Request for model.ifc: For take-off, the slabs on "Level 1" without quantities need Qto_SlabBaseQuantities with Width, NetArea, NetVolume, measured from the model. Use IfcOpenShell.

First a look at what the model holds.

```python
import ifcopenshell
import ifcopenshell.util.element
import ifcopenshell.util.unit

model = ifcopenshell.open("model.ifc")
print(model.schema)
for unit_type in ("LENGTHUNIT", "AREAUNIT", "VOLUMEUNIT"):
    print(unit_type, ifcopenshell.util.unit.calculate_unit_scale(model, unit_type))
storey = next(s for s in model.by_type("IfcBuildingStorey") if s.Name == "Level 1")
slabs = [e for e in ifcopenshell.util.element.get_decomposition(storey) if e.is_a("IfcSlab")]
for e in sorted(slabs, key=lambda e: e.id()):
    print(e.id(), e.is_a(), e.Name, list(ifcopenshell.util.element.get_psets(e, qtos_only=True)), sep=" | ")
```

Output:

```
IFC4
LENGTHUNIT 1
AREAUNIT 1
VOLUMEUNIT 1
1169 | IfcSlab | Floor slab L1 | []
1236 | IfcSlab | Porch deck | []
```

```python
import ifcopenshell
import ifcopenshell.api.pset
import ifcopenshell.geom
import ifcopenshell.util.element
import ifcopenshell.util.shape
import ifcopenshell.util.unit

model = ifcopenshell.open("model.ifc")
unit_scale = ifcopenshell.util.unit.calculate_unit_scale(model)
area_scale = ifcopenshell.util.unit.calculate_unit_scale(model, "AREAUNIT")
volume_scale = ifcopenshell.util.unit.calculate_unit_scale(model, "VOLUMEUNIT")
settings = ifcopenshell.geom.settings()

storey = next(s for s in model.by_type("IfcBuildingStorey") if s.Name == "Level 1")
slabs = [e for e in ifcopenshell.util.element.get_decomposition(storey) if e.is_a("IfcSlab")]

for e in sorted(slabs, key=lambda e: e.id()):
    if ifcopenshell.util.element.get_psets(e, qtos_only=True, should_inherit=False):
        continue
    # Geometry comes back in metres, in the element's own axes.
    shape = ifcopenshell.geom.create_shape(settings, e)
    values = {
        "Width": ifcopenshell.util.shape.get_z(shape.geometry) / unit_scale,
        "NetArea": ifcopenshell.util.shape.get_footprint_area(shape.geometry) / area_scale,
        "NetVolume": ifcopenshell.util.shape.get_volume(shape.geometry) / volume_scale,
    }
    qto = ifcopenshell.api.pset.add_qto(model, product=e, name="Qto_SlabBaseQuantities")
    ifcopenshell.api.pset.edit_qto(model, qto=qto, properties=values)
    print(e.id(), {k: round(v, 3) for k, v in values.items()})

model.write("model_edited.ifc")
```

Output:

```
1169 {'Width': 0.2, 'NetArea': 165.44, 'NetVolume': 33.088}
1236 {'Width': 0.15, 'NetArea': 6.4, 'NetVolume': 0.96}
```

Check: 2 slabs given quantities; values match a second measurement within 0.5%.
